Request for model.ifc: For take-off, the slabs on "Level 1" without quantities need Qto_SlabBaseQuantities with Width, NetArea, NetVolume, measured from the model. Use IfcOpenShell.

First a look at what the model holds.

```python
import ifcopenshell
import ifcopenshell.util.element
import ifcopenshell.util.unit

model = ifcopenshell.open("model.ifc")
print(model.schema)
for unit_type in ("LENGTHUNIT", "AREAUNIT", "VOLUMEUNIT"):
    print(unit_type, ifcopenshell.util.unit.calculate_unit_scale(model, unit_type))
storey = next(s for s in model.by_type("IfcBuildingStorey") if s.Name == "Level 1")
slabs = [e for e in ifcopenshell.util.element.get_decomposition(storey) if e.is_a("IfcSlab")]
for e in sorted(slabs, key=lambda e: e.id()):
    print(e.id(), e.is_a(), e.Name, list(ifcopenshell.util.element.get_psets(e, qtos_only=True)), sep=" | ")
```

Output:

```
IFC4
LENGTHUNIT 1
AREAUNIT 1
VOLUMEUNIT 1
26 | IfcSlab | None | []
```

```python
import ifcopenshell
import ifcopenshell.api.pset
import ifcopenshell.geom
import ifcopenshell.util.element
import ifcopenshell.util.shape
import ifcopenshell.util.unit

model = ifcopenshell.open("model.ifc")
unit_scale = ifcopenshell.util.unit.calculate_unit_scale(model)
area_scale = ifcopenshell.util.unit.calculate_unit_scale(model, "AREAUNIT")
volume_scale = ifcopenshell.util.unit.calculate_unit_scale(model, "VOLUMEUNIT")
settings = ifcopenshell.geom.settings()

storey = next(s for s in model.by_type("IfcBuildingStorey") if s.Name == "Level 1")
slabs = [e for e in ifcopenshell.util.element.get_decomposition(storey) if e.is_a("IfcSlab")]

for e in sorted(slabs, key=lambda e: e.id()):
    if ifcopenshell.util.element.get_psets(e, qtos_only=True, should_inherit=False):
        continue
    # Geometry comes back in metres, in the element's own axes.
    shape = ifcopenshell.geom.create_shape(settings, e)
    values = {
        "Width": ifcopenshell.util.shape.get_z(shape.geometry) / unit_scale,
        "NetArea": ifcopenshell.util.shape.get_footprint_area(shape.geometry) / area_scale,
        "NetVolume": ifcopenshell.util.shape.get_volume(shape.geometry) / volume_scale,
    }
    qto = ifcopenshell.api.pset.add_qto(model, product=e, name="Qto_SlabBaseQuantities")
    ifcopenshell.api.pset.edit_qto(model, qto=qto, properties=values)
    print(e.id(), {k: round(v, 3) for k, v in values.items()})

model.write("model-out.ifc")
```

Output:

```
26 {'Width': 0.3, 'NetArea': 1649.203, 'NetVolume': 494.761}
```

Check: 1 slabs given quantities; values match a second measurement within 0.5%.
